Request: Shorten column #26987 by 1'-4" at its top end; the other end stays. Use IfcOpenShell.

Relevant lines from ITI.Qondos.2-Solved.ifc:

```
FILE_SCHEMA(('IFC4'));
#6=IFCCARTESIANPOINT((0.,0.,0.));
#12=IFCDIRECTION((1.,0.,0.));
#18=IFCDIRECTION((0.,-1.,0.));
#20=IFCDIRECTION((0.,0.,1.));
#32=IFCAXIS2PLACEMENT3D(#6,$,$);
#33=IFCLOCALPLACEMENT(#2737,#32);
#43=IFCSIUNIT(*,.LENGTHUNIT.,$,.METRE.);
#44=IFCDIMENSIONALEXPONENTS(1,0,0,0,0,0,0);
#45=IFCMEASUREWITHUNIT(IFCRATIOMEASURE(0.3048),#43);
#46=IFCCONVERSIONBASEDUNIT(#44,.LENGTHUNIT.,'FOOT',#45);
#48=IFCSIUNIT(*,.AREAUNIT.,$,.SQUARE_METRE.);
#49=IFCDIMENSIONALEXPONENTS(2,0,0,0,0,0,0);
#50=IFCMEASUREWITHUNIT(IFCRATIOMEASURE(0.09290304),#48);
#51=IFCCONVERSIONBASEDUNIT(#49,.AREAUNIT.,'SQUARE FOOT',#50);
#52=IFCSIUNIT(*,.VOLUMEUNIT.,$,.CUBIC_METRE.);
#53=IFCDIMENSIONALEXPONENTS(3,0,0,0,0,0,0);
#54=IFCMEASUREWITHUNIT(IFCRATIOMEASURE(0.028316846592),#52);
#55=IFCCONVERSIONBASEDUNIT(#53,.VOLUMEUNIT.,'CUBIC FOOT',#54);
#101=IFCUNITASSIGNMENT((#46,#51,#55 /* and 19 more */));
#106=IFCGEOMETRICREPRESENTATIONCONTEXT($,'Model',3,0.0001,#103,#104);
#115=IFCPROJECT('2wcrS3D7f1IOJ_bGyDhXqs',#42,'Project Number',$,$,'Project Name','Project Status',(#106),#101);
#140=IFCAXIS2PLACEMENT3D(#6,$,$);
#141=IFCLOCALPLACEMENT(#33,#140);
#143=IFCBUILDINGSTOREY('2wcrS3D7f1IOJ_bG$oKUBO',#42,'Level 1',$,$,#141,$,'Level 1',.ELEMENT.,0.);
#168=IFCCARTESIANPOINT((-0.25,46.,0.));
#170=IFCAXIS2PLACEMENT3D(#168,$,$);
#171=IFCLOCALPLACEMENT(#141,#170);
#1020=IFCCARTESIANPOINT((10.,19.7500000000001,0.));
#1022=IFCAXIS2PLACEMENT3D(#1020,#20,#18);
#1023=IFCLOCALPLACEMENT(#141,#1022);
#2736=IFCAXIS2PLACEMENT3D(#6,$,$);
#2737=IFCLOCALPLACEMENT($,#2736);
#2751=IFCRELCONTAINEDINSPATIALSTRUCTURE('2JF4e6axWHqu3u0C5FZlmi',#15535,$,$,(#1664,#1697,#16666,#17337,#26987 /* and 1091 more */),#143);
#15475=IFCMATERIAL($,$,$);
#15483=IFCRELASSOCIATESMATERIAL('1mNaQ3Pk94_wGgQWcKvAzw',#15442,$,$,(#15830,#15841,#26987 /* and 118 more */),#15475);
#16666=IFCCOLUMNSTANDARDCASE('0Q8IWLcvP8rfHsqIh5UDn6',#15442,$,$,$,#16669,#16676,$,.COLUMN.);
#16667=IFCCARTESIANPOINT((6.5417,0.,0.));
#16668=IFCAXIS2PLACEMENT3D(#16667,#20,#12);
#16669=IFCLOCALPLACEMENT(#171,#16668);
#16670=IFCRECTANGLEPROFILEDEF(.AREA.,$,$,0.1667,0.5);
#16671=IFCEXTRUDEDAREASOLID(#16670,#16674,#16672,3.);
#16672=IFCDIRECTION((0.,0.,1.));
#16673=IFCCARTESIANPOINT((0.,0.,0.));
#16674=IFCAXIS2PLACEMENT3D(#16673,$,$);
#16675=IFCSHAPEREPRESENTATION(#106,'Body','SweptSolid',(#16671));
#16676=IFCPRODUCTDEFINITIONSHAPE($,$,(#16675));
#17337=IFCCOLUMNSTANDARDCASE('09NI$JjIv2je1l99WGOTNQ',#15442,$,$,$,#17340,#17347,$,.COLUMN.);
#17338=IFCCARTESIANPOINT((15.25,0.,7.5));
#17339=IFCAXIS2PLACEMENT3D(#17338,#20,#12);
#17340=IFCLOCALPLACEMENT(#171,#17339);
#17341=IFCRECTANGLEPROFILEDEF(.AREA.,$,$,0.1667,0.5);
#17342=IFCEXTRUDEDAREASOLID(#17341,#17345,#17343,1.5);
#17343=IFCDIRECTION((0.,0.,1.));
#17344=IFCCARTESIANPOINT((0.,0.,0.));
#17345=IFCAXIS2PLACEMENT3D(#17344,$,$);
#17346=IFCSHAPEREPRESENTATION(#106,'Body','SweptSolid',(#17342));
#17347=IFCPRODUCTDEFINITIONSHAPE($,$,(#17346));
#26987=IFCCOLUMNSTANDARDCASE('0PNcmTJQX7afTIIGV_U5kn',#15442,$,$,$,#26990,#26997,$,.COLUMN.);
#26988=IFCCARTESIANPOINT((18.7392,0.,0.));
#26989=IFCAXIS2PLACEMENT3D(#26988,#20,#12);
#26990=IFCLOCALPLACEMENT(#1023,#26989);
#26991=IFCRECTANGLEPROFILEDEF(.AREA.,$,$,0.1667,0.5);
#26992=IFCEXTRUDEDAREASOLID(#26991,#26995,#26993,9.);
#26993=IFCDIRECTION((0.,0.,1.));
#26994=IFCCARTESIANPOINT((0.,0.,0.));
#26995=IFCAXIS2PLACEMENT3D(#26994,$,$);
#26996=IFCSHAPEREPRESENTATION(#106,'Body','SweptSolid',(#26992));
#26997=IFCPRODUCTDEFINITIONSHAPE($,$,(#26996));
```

```python
import ifcopenshell
import ifcopenshell.util.unit

model = ifcopenshell.open("ITI.Qondos.2-Solved.ifc")
unit_scale = ifcopenshell.util.unit.calculate_unit_scale(model)

member = model.by_id(26987)
change = -16 * 0.0254 / unit_scale

# The extrusion runs towards the end named, so only its depth changes.
body = next(r for r in member.Representation.Representations if r.RepresentationIdentifier == "Body")
solid = body.Items[0]
old_length = solid.Depth
solid.Depth += change

print(f"length {old_length:g} -> {solid.Depth:g}")

model.write("ITI.Qondos.2-Solved_edited.ifc")
```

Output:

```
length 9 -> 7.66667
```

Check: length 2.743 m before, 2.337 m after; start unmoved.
